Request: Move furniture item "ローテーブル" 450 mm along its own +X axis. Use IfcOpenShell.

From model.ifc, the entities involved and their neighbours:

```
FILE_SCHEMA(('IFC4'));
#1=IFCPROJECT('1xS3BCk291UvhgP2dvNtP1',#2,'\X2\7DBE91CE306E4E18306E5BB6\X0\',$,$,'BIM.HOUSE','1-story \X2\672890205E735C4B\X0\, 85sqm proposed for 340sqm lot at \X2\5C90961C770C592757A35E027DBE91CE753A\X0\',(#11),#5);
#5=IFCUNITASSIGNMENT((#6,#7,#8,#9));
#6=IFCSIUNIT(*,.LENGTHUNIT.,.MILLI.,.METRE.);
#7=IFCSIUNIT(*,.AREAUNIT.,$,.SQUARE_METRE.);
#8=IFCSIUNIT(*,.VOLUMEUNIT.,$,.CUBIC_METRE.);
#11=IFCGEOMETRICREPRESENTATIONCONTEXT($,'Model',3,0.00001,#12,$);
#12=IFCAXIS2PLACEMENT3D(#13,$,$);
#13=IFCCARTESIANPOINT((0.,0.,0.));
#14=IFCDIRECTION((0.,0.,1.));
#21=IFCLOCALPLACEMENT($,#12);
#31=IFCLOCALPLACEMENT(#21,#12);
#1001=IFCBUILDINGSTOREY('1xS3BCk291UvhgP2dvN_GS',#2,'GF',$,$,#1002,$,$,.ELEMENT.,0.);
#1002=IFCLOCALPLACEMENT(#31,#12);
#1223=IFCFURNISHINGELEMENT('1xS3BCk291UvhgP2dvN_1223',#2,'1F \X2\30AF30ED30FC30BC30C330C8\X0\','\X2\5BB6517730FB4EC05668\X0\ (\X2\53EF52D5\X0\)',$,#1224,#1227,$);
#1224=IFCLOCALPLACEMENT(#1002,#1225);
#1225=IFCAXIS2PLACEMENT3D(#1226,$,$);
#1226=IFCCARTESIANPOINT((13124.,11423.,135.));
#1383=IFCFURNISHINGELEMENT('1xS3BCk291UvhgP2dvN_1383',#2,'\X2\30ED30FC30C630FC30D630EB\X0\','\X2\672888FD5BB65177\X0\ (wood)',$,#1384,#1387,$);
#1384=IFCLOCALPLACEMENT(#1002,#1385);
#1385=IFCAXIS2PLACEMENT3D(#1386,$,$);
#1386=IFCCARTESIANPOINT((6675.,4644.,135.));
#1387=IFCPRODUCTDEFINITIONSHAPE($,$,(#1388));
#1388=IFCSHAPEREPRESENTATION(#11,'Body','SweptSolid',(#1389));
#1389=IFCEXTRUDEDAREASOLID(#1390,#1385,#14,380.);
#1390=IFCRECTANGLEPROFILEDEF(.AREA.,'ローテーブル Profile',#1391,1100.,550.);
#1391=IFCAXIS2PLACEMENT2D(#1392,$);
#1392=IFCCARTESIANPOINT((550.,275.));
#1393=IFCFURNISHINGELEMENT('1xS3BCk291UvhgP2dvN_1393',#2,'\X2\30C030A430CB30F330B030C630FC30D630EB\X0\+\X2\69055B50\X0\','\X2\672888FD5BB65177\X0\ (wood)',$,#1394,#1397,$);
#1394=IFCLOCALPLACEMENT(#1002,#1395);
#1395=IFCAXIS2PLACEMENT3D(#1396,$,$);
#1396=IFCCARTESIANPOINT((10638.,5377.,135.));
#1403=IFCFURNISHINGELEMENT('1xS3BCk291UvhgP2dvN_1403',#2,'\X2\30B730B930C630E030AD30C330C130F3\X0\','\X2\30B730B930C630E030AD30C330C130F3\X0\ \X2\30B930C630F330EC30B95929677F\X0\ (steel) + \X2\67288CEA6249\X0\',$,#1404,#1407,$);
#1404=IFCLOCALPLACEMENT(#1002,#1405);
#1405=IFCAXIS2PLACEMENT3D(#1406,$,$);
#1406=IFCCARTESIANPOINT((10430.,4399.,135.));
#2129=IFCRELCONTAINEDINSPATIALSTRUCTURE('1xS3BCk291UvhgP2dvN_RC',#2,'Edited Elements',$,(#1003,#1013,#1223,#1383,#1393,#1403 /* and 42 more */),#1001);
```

```python
import ifcopenshell
import ifcopenshell.api.geometry
import ifcopenshell.util.placement
import ifcopenshell.util.unit

model = ifcopenshell.open("model.ifc")
unit_scale = ifcopenshell.util.unit.calculate_unit_scale(model)

item = model.by_guid("1xS3BCk291UvhgP2dvN_1383")
matrix = ifcopenshell.util.placement.get_local_placement(item.ObjectPlacement)
matrix[:3, 3] += matrix[:3, 0] * 0.45 / unit_scale
ifcopenshell.api.geometry.edit_object_placement(model, product=item, matrix=matrix, is_si=False)

print(ifcopenshell.util.placement.get_local_placement(item.ObjectPlacement).round(3) + 0.0)

model.write("model-out.ifc")
```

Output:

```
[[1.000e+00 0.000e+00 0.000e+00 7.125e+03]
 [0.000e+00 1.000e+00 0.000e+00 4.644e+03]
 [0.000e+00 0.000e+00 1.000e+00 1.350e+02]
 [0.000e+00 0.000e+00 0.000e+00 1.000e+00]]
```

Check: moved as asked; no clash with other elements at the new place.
